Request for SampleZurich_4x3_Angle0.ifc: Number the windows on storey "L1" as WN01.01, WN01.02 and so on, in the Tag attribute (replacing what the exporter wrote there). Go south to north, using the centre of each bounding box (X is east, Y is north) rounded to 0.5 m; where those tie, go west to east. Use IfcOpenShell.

First a look at what the model holds.

```python
import ifcopenshell
import ifcopenshell.util.element
import ifcopenshell.util.placement

model = ifcopenshell.open("SampleZurich_4x3_Angle0.ifc")
print(model.schema)
storey = next(s for s in model.by_type("IfcBuildingStorey") if s.Name == "L1")
windows = [e for e in ifcopenshell.util.element.get_decomposition(storey) if e.is_a("IfcWindow")]
for e in sorted(windows, key=lambda e: e.id()):
    origin = ifcopenshell.util.placement.get_local_placement(e.ObjectPlacement)[:3, 3]
    print(e.id(), e.Tag, e.Name, origin.round(2) + 0.0, sep=" | ")
```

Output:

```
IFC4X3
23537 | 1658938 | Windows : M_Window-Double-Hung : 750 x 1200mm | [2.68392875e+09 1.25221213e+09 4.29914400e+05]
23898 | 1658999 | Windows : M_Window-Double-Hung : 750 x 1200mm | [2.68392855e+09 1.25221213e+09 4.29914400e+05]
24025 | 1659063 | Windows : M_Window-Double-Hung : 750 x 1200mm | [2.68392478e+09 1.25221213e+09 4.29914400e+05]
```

```python
import ifcopenshell
import ifcopenshell.geom
import ifcopenshell.util.element
import ifcopenshell.util.shape

model = ifcopenshell.open("SampleZurich_4x3_Angle0.ifc")
settings = ifcopenshell.geom.settings()
settings.set("use-world-coords", True)


def centre(element):
    shape = ifcopenshell.geom.create_shape(settings, element)
    return ifcopenshell.util.shape.get_bbox_centroid(shape.geometry)


storey = next(s for s in model.by_type("IfcBuildingStorey") if s.Name == "L1")
windows = [e for e in ifcopenshell.util.element.get_decomposition(storey) if e.is_a("IfcWindow")]

# Insertion points can sit at a corner or the storey origin, so sort by the geometry (in metres).
centres = {e: centre(e) for e in windows}
windows.sort(key=lambda e: (round(centres[e][1] / 0.5), centres[e][0]))

for i, e in enumerate(windows, start=1):
    number = f"WN01.{i:02d}"
    e.Tag = number
    print(e.id(), number)

model.write("SampleZurich_4x3_Angle0_updated.ifc")
```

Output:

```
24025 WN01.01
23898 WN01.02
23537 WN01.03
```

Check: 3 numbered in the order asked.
